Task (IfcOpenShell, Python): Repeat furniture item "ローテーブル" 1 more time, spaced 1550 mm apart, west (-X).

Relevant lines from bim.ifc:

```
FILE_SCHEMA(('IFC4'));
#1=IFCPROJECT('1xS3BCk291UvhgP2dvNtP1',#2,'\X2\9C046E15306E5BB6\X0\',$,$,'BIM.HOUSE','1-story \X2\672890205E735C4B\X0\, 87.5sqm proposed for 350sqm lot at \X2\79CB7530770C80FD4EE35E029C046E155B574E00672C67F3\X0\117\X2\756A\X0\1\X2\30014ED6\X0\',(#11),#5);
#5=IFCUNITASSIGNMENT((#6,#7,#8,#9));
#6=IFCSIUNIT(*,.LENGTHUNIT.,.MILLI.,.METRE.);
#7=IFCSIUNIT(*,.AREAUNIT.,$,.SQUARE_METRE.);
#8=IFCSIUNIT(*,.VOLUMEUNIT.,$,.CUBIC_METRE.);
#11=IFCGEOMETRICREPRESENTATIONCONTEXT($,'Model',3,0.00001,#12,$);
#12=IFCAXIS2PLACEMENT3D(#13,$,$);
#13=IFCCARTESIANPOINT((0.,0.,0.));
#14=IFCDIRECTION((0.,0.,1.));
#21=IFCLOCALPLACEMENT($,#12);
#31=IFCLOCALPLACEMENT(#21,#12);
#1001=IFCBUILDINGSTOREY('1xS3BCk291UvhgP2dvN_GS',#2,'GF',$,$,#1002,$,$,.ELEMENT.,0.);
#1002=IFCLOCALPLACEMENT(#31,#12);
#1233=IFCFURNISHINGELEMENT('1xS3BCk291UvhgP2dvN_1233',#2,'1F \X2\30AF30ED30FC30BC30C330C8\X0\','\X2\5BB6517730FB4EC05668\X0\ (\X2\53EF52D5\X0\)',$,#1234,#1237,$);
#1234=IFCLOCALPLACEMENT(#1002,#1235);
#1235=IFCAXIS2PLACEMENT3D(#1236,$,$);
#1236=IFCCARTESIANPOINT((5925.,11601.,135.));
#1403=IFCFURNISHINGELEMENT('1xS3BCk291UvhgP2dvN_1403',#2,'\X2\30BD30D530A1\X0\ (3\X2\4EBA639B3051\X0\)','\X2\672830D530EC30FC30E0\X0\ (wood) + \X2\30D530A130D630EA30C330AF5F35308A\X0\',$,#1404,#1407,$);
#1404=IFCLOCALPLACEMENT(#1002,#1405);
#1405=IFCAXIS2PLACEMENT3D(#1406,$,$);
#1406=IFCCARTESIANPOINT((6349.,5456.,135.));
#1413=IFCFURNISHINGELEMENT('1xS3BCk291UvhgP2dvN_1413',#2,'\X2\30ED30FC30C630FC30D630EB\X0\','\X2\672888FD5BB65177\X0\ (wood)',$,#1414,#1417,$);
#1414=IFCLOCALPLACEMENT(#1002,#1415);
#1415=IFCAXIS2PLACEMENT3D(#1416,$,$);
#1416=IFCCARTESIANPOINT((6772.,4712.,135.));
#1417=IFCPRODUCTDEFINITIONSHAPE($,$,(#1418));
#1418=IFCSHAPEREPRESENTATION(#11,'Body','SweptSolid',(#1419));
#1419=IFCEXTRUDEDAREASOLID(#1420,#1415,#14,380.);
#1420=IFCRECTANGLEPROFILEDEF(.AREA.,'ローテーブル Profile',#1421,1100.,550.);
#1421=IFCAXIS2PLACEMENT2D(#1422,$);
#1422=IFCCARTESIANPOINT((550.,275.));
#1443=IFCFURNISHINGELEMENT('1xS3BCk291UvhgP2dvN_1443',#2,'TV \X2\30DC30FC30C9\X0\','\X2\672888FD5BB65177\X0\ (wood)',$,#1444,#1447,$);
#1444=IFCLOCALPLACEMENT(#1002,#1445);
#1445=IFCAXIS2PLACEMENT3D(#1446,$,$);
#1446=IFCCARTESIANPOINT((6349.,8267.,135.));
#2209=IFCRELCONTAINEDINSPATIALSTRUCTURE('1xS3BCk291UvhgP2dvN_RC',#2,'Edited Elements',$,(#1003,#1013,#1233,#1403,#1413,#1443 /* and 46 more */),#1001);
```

```python
import numpy as np
import ifcopenshell
import ifcopenshell.api.geometry
import ifcopenshell.api.root
import ifcopenshell.util.element
import ifcopenshell.util.placement

model = ifcopenshell.open("bim.ifc")


def reuse_history(source, copy):
    """copy_class also copies each property set's owner history, people and application; keep the originals."""
    for rel in copy.IsDefinedBy:
        if rel.is_a("IfcRelDefinesByProperties") and (history := rel.RelatingPropertyDefinition.OwnerHistory):
            rel.RelatingPropertyDefinition.OwnerHistory = source.OwnerHistory
            ifcopenshell.util.element.remove_deep2(model, history)


source = model.by_guid("1xS3BCk291UvhgP2dvN_1413")
base = ifcopenshell.util.placement.get_local_placement(source.ObjectPlacement)
step = np.array([-1.0, 0.0, 0.0]) * 1550.0

for i in range(1, 2):
    copy = ifcopenshell.api.root.copy_class(model, product=source)
    copy.Representation = ifcopenshell.util.element.copy_deep(
        model, source.Representation, exclude=["IfcGeometricRepresentationContext", "IfcRepresentationMap"]
    )
    reuse_history(source, copy)
    matrix = base.copy()
    matrix[:3, 3] += i * step
    print("added at", matrix[:3, 3].round(3) + 0.0)
    ifcopenshell.api.geometry.edit_object_placement(model, product=copy, matrix=matrix, is_si=False)

model.write("bim_updated.ifc")
```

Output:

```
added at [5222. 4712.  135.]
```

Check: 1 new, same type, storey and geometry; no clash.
